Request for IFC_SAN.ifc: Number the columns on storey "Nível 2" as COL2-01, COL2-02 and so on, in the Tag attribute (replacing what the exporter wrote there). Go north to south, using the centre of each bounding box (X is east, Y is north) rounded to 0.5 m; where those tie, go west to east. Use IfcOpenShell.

First a look at what the model holds.

```python
import ifcopenshell
import ifcopenshell.util.element
import ifcopenshell.util.placement

model = ifcopenshell.open("IFC_SAN.ifc")
print(model.schema)
storey = next(s for s in model.by_type("IfcBuildingStorey") if s.Name == "Nível 2")
columns = [e for e in ifcopenshell.util.element.get_decomposition(storey) if e.is_a("IfcColumn")]
for e in sorted(columns, key=lambda e: e.id()):
    origin = ifcopenshell.util.placement.get_local_placement(e.ObjectPlacement)[:3, 3]
    print(e.id(), e.Tag, e.Name, origin.round(2) + 0.0, sep=" | ")
```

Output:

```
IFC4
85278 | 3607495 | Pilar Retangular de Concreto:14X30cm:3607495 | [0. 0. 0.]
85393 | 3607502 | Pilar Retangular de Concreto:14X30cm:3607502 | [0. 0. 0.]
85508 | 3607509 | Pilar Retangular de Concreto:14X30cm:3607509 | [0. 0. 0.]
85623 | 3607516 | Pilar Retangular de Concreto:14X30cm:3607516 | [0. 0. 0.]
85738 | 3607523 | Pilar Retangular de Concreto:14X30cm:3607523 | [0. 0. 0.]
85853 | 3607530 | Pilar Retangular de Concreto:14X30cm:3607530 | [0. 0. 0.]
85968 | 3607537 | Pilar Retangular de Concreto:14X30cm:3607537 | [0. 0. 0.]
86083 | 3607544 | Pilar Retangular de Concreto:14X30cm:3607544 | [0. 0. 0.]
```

```python
import ifcopenshell
import ifcopenshell.geom
import ifcopenshell.util.element
import ifcopenshell.util.shape

model = ifcopenshell.open("IFC_SAN.ifc")
settings = ifcopenshell.geom.settings()
settings.set("use-world-coords", True)


def centre(element):
    shape = ifcopenshell.geom.create_shape(settings, element)
    return ifcopenshell.util.shape.get_bbox_centroid(shape.geometry)


storey = next(s for s in model.by_type("IfcBuildingStorey") if s.Name == "Nível 2")
columns = [e for e in ifcopenshell.util.element.get_decomposition(storey) if e.is_a("IfcColumn")]

# Insertion points can sit at a corner or the storey origin, so sort by the geometry (in metres).
centres = {e: centre(e) for e in columns}
columns.sort(key=lambda e: (-round(centres[e][1] / 0.5), centres[e][0]))

for i, e in enumerate(columns, start=1):
    number = f"COL2-{i:02d}"
    e.Tag = number
    print(e.id(), number)

model.write("IFC_SAN-out.ifc")
```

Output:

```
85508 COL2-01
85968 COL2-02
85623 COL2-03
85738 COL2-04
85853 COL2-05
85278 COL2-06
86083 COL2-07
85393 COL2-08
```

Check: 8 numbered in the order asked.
